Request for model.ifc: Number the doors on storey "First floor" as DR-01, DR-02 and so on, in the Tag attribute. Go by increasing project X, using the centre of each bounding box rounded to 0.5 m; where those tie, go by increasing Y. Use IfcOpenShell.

First a look at what the model holds.

```python
import ifcopenshell
import ifcopenshell.util.element
import ifcopenshell.util.placement

model = ifcopenshell.open("model.ifc")
print(model.schema)
storey = next(s for s in model.by_type("IfcBuildingStorey") if s.Name == "First floor")
doors = [e for e in ifcopenshell.util.element.get_decomposition(storey) if e.is_a("IfcDoor")]
for e in sorted(doors, key=lambda e: e.id()):
    origin = ifcopenshell.util.placement.get_local_placement(e.ObjectPlacement)[:3, 3]
    print(e.id(), e.Tag, e.Name, origin.round(2) + 0.0, sep=" | ")
```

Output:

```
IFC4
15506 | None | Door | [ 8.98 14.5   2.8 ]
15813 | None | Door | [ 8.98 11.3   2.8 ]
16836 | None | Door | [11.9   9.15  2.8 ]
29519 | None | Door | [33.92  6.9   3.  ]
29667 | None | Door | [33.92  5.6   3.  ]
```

```python
import ifcopenshell
import ifcopenshell.geom
import ifcopenshell.util.element
import ifcopenshell.util.shape

model = ifcopenshell.open("model.ifc")
settings = ifcopenshell.geom.settings()
settings.set("use-world-coords", True)


def centre(element):
    shape = ifcopenshell.geom.create_shape(settings, element)
    return ifcopenshell.util.shape.get_bbox_centroid(shape.geometry)


storey = next(s for s in model.by_type("IfcBuildingStorey") if s.Name == "First floor")
doors = [e for e in ifcopenshell.util.element.get_decomposition(storey) if e.is_a("IfcDoor")]

# Insertion points can sit at a corner or the storey origin, so sort by the geometry (in metres).
centres = {e: centre(e) for e in doors}
doors.sort(key=lambda e: (round(centres[e][0] / 0.5), centres[e][1]))

for i, e in enumerate(doors, start=1):
    number = f"DR-{i:02d}"
    e.Tag = number
    print(e.id(), number)

model.write("model_edited.ifc")
```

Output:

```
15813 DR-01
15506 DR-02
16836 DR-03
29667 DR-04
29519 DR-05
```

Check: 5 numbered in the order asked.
